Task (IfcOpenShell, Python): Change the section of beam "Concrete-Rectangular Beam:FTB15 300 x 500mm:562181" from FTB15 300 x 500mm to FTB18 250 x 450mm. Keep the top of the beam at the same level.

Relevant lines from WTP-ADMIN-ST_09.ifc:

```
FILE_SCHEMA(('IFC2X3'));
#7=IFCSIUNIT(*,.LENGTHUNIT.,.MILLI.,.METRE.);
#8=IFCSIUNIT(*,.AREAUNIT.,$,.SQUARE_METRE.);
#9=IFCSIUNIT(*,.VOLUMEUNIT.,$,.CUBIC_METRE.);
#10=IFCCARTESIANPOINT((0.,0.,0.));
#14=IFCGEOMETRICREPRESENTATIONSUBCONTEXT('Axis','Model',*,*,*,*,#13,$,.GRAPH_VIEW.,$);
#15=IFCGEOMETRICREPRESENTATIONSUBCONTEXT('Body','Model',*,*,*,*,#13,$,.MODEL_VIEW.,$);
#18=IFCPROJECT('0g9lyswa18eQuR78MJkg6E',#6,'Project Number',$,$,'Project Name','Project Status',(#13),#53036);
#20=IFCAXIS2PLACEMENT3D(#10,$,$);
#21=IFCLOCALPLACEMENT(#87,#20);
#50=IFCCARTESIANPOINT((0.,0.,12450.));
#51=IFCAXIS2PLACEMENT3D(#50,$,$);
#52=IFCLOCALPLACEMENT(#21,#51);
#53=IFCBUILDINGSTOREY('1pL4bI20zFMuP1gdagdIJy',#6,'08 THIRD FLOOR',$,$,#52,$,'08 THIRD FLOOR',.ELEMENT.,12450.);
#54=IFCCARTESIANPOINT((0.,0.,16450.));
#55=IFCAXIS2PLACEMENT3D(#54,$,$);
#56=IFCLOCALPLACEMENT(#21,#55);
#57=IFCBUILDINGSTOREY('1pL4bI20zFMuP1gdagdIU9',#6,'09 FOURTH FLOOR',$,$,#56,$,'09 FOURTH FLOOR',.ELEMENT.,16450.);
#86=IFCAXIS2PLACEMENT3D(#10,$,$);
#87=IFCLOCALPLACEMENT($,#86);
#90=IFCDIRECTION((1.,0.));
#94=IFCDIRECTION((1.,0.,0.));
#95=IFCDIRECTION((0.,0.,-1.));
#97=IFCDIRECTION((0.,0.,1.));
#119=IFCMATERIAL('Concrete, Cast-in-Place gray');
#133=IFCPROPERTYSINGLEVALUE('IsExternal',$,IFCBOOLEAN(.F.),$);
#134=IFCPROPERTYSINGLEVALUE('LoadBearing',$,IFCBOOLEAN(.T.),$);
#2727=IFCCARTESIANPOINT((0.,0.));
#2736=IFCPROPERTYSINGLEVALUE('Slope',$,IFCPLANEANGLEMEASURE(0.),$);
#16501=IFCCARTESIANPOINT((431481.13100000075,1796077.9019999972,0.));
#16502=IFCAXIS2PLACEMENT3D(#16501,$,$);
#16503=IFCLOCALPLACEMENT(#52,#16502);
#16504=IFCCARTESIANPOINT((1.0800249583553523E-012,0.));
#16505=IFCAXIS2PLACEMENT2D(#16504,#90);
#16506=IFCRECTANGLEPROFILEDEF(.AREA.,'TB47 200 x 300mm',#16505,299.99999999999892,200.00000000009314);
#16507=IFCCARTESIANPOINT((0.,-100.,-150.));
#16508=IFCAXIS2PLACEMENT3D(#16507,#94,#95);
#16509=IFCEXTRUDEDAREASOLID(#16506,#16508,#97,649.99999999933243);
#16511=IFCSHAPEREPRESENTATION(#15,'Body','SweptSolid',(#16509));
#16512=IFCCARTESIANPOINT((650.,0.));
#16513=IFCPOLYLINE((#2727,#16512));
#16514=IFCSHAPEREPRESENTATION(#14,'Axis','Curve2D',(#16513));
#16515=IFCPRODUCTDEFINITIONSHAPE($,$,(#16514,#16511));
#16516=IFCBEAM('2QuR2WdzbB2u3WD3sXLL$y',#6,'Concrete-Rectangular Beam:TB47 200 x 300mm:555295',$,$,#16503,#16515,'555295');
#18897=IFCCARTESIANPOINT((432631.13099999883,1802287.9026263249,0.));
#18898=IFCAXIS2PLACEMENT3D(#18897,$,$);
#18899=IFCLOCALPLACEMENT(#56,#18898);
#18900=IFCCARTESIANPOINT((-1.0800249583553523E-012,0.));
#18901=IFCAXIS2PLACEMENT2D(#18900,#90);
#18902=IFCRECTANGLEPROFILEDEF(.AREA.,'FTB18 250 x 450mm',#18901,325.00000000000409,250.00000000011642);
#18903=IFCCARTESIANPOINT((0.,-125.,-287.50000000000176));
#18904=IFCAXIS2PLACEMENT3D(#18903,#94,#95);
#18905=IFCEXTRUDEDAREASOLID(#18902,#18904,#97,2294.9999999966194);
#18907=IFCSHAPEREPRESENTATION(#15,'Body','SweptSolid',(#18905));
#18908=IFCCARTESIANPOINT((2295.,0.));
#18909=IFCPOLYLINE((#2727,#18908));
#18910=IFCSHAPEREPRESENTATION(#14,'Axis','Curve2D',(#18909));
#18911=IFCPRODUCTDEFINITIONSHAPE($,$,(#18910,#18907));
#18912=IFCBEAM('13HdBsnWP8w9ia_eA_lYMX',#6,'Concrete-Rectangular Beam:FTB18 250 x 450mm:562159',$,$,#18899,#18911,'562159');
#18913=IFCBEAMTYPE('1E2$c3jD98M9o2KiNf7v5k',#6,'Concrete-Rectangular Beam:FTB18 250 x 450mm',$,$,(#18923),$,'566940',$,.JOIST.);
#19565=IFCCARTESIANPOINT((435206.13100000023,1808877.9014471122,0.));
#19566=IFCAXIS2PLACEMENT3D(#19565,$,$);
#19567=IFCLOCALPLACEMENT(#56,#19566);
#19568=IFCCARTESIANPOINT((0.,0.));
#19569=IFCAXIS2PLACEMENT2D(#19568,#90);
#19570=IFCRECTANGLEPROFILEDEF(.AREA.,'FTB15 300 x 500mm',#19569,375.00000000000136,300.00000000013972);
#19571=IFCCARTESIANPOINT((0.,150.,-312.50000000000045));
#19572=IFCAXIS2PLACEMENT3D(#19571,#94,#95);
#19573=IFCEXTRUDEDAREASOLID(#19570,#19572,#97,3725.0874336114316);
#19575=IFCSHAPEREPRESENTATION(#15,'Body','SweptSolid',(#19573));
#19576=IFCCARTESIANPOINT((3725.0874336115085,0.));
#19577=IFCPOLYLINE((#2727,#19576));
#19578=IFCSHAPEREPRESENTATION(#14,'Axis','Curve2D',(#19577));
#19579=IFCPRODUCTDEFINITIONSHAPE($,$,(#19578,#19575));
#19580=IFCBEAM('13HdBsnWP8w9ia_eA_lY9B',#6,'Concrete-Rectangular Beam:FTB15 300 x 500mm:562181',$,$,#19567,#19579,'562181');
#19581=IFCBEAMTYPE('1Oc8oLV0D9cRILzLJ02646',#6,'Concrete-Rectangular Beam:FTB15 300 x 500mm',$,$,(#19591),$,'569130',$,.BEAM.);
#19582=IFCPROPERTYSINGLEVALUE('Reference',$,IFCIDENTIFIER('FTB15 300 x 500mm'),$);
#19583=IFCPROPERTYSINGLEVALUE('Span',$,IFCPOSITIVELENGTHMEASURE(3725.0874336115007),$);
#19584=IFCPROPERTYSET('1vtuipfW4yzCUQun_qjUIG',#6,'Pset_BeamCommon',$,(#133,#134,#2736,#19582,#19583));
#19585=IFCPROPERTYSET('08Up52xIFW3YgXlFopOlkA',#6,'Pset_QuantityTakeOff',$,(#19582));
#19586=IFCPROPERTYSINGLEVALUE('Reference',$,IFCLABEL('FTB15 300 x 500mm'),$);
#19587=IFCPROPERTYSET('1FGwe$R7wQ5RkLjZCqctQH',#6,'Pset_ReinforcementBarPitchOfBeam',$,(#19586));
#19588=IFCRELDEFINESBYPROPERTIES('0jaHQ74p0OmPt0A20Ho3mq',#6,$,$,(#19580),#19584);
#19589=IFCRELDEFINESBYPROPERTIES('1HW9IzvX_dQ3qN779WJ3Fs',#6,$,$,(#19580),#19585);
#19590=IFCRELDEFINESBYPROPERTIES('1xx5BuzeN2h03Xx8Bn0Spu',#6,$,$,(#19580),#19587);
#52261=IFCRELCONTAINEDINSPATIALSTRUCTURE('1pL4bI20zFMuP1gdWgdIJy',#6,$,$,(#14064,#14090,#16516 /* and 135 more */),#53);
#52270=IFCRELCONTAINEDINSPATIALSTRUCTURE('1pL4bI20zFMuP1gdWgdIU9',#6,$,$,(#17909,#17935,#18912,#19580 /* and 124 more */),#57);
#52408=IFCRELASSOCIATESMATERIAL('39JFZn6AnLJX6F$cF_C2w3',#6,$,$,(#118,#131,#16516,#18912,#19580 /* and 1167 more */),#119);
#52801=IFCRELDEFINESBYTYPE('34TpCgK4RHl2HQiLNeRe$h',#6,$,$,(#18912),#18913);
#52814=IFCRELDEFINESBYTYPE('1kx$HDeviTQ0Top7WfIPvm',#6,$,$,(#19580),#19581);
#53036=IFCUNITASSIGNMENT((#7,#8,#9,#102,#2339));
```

```python
import ifcopenshell
import ifcopenshell.api.pset
import ifcopenshell.api.type
import ifcopenshell.util.element
import ifcopenshell.util.representation

model = ifcopenshell.open("WTP-ADMIN-ST_09.ifc")

member = model.by_guid("13HdBsnWP8w9ia_eA_lY9B")
source = next(p for p in model.by_type("IfcRectangleProfileDef") if p.ProfileName == "FTB18 250 x 450mm")

body = ifcopenshell.util.representation.get_representation(member, "Model", "Body")
solid = body.Items[0]
old_profile = solid.SweptArea

# Copy the section's sizes but keep this member's own profile position.
profile = ifcopenshell.util.element.copy(model, source)
# Profiles are centred, so shift by half the change in depth to hold the top.
shift = (old_profile.XDim - profile.XDim) / 2
x, y = old_profile.Position.Location.Coordinates
up = (-1.0, 0.0)  # upwards, in the solid's own plane
location = model.createIfcCartesianPoint((x + up[0] * shift, y + up[1] * shift))
profile.Position = model.createIfcAxis2Placement2D(location, old_profile.Position.RefDirection)
solid.SweptArea = profile
if not model.get_total_inverses(old_profile):
    ifcopenshell.util.element.remove_deep2(model, old_profile)

new_type = model.by_guid("1E2$c3jD98M9o2KiNf7v5k")
ifcopenshell.api.type.assign_type(
    model, related_objects=[member], relating_type=new_type, should_map_representations=False
)
member.Name = member.Name.replace("FTB15 300 x 500mm", "FTB18 250 x 450mm")
pset = model.by_id(ifcopenshell.util.element.get_pset(member, "Pset_BeamCommon", should_inherit=False)["id"])
ifcopenshell.api.pset.edit_pset(model, pset=pset, properties={"Reference": "FTB18 250 x 450mm"})
pset = model.by_id(ifcopenshell.util.element.get_pset(member, "Pset_QuantityTakeOff", should_inherit=False)["id"])
ifcopenshell.api.pset.edit_pset(model, pset=pset, properties={"Reference": "FTB18 250 x 450mm"})
pset = model.by_id(ifcopenshell.util.element.get_pset(member, "Pset_ReinforcementBarPitchOfBeam", should_inherit=False)["id"])
ifcopenshell.api.pset.edit_pset(model, pset=pset, properties={"Reference": "FTB18 250 x 450mm"})

print(solid.SweptArea)

model.write("WTP-ADMIN-ST_09_rev.ifc")
```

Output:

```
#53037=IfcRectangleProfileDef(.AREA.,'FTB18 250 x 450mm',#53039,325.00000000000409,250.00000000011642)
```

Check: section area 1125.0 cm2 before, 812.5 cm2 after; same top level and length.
